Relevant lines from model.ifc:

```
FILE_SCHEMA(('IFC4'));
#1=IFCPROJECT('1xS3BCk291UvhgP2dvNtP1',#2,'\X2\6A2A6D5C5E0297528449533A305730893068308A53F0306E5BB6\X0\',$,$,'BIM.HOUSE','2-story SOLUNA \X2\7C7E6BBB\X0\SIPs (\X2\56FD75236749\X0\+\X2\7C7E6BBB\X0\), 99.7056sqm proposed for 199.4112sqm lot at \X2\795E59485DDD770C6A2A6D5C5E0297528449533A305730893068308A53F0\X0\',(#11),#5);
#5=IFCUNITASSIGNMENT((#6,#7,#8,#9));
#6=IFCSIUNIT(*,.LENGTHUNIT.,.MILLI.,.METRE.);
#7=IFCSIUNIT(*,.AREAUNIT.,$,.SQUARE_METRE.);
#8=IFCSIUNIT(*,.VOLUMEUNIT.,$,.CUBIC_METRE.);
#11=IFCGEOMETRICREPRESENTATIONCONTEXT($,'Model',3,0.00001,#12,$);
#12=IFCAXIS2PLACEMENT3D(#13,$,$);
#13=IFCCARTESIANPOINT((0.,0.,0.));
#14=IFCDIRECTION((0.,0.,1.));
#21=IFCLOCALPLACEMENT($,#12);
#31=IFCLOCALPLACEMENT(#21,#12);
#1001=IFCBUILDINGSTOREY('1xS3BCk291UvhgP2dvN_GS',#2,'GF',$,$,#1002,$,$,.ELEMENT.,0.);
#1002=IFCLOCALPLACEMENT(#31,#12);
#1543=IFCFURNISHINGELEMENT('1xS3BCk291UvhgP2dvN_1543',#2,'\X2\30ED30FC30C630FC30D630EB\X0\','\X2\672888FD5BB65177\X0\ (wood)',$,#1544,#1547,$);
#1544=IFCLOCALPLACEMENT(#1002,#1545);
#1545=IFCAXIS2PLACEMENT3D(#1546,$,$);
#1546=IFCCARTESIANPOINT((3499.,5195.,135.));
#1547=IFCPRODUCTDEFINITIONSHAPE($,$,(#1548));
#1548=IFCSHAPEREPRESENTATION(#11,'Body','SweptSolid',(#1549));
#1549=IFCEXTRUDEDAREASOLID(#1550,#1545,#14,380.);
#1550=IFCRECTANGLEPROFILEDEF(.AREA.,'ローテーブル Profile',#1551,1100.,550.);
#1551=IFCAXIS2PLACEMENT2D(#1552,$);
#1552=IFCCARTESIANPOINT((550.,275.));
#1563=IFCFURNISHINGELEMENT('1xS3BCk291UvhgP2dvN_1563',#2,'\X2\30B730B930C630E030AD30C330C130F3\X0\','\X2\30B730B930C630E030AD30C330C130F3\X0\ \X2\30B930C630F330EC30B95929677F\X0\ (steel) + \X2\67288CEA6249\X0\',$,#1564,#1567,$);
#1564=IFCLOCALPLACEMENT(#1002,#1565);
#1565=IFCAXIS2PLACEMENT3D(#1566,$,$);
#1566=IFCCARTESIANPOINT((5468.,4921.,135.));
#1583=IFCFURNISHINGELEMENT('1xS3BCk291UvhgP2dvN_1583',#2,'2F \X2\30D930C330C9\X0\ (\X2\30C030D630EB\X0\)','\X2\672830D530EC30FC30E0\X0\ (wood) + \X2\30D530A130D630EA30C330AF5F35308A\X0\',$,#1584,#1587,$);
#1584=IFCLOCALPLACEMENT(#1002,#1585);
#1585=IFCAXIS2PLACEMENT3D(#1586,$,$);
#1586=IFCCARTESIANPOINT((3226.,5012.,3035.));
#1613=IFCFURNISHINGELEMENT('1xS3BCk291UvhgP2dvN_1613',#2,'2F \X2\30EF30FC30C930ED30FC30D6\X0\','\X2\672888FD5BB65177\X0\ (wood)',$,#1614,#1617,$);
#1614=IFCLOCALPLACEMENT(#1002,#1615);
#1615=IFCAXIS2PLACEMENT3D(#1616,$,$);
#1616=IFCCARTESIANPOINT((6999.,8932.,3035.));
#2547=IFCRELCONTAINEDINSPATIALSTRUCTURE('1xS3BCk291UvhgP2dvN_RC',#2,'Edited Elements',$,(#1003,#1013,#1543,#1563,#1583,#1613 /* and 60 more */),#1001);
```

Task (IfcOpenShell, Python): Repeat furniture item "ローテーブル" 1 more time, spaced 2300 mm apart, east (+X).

```python
import numpy as np
import ifcopenshell
import ifcopenshell.api.geometry
import ifcopenshell.api.root
import ifcopenshell.util.element
import ifcopenshell.util.placement
import ifcopenshell.util.unit

model = ifcopenshell.open("model.ifc")
unit_scale = ifcopenshell.util.unit.calculate_unit_scale(model)


def reuse_history(source, copy):
    """copy_class also copies each property set's owner history, people and application; keep the originals."""
    for rel in copy.IsDefinedBy:
        if rel.is_a("IfcRelDefinesByProperties") and (history := rel.RelatingPropertyDefinition.OwnerHistory):
            rel.RelatingPropertyDefinition.OwnerHistory = source.OwnerHistory
            ifcopenshell.util.element.remove_deep2(model, history)


source = model.by_guid("1xS3BCk291UvhgP2dvN_1543")
base = ifcopenshell.util.placement.get_local_placement(source.ObjectPlacement)
step = np.array([1.0, 0.0, 0.0]) * 2.3 / unit_scale

for i in range(1, 2):
    copy = ifcopenshell.api.root.copy_class(model, product=source)
    copy.Representation = ifcopenshell.util.element.copy_deep(
        model, source.Representation, exclude=["IfcGeometricRepresentationContext", "IfcRepresentationMap"]
    )
    reuse_history(source, copy)
    matrix = base.copy()
    matrix[:3, 3] += i * step
    print("added at", matrix[:3, 3].round(3) + 0.0)
    ifcopenshell.api.geometry.edit_object_placement(model, product=copy, matrix=matrix, is_si=False)

model.write("model_edited.ifc")
```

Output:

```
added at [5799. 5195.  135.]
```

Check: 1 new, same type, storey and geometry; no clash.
